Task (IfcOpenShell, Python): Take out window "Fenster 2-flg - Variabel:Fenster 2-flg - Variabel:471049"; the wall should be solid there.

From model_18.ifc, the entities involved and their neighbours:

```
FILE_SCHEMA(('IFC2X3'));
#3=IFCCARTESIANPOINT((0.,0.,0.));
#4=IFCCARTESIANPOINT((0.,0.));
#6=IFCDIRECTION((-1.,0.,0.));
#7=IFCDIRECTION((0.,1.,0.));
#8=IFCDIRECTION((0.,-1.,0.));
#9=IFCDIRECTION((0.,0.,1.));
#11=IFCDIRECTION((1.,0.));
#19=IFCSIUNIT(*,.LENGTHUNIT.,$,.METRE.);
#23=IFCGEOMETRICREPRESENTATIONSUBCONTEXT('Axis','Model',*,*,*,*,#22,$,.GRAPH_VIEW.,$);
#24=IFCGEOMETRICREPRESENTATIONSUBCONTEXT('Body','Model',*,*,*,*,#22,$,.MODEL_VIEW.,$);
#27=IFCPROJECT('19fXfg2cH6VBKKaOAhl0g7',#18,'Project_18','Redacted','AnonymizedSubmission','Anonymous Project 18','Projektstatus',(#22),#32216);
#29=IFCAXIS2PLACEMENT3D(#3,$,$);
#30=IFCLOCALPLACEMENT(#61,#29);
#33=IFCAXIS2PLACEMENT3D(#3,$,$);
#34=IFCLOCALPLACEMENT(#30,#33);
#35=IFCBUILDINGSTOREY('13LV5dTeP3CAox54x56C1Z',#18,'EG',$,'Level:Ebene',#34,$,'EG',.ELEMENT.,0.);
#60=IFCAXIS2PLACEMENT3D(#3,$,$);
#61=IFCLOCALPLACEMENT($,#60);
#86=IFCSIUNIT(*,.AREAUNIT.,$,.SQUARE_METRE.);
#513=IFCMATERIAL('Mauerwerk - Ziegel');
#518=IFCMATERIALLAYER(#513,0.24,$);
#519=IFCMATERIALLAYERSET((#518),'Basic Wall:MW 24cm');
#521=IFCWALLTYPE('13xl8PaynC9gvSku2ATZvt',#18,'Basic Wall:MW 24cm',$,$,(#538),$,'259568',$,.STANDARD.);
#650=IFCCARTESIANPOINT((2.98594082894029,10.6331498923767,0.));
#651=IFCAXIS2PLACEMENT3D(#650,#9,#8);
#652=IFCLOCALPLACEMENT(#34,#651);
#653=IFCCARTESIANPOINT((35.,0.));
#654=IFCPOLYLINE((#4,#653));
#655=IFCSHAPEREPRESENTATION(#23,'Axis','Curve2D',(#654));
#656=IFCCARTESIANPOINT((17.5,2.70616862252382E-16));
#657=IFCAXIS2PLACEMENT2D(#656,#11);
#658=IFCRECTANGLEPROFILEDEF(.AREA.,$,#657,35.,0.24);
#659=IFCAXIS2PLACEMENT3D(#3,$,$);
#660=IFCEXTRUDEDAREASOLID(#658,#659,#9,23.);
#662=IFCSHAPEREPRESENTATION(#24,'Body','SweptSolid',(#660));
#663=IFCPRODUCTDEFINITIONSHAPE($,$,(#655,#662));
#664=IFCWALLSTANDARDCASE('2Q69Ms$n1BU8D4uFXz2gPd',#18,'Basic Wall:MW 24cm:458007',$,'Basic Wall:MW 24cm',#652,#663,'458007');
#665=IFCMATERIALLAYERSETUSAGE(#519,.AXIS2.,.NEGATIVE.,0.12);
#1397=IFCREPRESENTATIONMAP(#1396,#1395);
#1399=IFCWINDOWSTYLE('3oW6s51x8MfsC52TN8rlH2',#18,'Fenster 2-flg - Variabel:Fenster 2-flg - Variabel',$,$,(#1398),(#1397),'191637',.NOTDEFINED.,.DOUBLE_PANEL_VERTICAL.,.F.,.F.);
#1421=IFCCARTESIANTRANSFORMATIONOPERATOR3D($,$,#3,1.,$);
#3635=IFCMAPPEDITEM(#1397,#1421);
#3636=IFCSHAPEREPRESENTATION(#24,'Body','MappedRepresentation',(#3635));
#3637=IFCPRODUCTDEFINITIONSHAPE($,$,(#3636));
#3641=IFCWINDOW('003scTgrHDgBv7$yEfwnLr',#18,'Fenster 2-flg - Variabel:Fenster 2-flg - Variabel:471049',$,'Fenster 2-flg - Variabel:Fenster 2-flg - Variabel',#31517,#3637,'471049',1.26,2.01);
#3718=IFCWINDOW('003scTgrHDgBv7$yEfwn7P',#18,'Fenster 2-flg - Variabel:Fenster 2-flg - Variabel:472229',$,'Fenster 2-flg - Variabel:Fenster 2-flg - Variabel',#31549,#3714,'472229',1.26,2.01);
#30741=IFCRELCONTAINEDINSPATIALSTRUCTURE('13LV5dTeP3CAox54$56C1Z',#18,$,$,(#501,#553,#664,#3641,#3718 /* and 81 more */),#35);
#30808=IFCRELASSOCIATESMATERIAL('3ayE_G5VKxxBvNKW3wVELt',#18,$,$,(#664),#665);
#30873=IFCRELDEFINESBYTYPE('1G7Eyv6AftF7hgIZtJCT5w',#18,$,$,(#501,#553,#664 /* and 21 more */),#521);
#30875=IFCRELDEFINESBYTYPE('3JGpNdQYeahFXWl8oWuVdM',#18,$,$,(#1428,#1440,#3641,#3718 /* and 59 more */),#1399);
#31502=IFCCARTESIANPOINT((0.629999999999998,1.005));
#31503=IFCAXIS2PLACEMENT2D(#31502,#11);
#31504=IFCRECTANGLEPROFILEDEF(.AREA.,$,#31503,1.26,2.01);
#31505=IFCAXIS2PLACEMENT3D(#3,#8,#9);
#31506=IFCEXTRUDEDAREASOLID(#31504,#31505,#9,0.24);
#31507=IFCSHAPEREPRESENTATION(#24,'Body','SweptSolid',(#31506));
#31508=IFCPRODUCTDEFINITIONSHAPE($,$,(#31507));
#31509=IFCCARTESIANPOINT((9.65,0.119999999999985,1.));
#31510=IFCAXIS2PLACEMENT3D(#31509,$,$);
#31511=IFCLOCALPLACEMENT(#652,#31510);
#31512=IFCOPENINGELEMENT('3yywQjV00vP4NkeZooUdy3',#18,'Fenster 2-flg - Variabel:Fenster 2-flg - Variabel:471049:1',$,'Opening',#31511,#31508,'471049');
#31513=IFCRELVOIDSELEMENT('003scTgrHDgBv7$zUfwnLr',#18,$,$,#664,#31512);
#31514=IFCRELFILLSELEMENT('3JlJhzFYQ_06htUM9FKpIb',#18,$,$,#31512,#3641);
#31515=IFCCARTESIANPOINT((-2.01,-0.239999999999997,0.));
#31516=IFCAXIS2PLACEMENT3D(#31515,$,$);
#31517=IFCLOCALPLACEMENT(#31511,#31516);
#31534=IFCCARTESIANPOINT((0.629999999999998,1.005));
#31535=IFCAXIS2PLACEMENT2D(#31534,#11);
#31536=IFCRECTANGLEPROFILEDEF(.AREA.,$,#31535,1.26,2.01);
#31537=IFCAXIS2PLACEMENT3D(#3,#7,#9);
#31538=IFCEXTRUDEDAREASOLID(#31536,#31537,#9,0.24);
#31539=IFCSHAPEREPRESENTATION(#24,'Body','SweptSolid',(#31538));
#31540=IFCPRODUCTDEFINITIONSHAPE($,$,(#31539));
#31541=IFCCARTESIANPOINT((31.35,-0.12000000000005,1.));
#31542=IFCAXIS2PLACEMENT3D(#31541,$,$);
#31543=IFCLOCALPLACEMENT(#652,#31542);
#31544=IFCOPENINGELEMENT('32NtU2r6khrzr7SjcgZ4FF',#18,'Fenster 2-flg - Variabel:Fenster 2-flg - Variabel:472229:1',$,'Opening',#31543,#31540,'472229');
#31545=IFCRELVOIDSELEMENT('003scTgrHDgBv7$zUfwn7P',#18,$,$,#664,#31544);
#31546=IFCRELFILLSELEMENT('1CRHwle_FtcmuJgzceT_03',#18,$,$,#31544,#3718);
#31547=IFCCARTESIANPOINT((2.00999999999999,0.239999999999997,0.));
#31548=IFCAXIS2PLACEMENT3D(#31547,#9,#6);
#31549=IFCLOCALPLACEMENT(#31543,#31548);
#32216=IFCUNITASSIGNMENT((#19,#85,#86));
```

```python
import ifcopenshell
import ifcopenshell.api.feature
import ifcopenshell.api.root
import ifcopenshell.geom
import ifcopenshell.util.shape

model = ifcopenshell.open("model_18.ifc")
settings = ifcopenshell.geom.settings()


def volume(element):
    """Net volume in cubic metres, openings subtracted."""
    shape = ifcopenshell.geom.create_shape(settings, element)
    return ifcopenshell.util.shape.get_volume(shape.geometry)


window = model.by_id(3641)
opening = window.FillsVoids[0].RelatingOpeningElement
wall = opening.VoidsElements[0].RelatingBuildingElement
before = volume(wall)

ifcopenshell.api.root.remove_product(model, product=window)
ifcopenshell.api.feature.remove_feature(model, feature=opening)

after = volume(wall)

print(f"wall volume {before:.3f} -> {after:.3f} m3")

model.write("model_18_edited.ifc")
```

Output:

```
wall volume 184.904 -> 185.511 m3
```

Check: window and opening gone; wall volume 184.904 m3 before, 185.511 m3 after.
